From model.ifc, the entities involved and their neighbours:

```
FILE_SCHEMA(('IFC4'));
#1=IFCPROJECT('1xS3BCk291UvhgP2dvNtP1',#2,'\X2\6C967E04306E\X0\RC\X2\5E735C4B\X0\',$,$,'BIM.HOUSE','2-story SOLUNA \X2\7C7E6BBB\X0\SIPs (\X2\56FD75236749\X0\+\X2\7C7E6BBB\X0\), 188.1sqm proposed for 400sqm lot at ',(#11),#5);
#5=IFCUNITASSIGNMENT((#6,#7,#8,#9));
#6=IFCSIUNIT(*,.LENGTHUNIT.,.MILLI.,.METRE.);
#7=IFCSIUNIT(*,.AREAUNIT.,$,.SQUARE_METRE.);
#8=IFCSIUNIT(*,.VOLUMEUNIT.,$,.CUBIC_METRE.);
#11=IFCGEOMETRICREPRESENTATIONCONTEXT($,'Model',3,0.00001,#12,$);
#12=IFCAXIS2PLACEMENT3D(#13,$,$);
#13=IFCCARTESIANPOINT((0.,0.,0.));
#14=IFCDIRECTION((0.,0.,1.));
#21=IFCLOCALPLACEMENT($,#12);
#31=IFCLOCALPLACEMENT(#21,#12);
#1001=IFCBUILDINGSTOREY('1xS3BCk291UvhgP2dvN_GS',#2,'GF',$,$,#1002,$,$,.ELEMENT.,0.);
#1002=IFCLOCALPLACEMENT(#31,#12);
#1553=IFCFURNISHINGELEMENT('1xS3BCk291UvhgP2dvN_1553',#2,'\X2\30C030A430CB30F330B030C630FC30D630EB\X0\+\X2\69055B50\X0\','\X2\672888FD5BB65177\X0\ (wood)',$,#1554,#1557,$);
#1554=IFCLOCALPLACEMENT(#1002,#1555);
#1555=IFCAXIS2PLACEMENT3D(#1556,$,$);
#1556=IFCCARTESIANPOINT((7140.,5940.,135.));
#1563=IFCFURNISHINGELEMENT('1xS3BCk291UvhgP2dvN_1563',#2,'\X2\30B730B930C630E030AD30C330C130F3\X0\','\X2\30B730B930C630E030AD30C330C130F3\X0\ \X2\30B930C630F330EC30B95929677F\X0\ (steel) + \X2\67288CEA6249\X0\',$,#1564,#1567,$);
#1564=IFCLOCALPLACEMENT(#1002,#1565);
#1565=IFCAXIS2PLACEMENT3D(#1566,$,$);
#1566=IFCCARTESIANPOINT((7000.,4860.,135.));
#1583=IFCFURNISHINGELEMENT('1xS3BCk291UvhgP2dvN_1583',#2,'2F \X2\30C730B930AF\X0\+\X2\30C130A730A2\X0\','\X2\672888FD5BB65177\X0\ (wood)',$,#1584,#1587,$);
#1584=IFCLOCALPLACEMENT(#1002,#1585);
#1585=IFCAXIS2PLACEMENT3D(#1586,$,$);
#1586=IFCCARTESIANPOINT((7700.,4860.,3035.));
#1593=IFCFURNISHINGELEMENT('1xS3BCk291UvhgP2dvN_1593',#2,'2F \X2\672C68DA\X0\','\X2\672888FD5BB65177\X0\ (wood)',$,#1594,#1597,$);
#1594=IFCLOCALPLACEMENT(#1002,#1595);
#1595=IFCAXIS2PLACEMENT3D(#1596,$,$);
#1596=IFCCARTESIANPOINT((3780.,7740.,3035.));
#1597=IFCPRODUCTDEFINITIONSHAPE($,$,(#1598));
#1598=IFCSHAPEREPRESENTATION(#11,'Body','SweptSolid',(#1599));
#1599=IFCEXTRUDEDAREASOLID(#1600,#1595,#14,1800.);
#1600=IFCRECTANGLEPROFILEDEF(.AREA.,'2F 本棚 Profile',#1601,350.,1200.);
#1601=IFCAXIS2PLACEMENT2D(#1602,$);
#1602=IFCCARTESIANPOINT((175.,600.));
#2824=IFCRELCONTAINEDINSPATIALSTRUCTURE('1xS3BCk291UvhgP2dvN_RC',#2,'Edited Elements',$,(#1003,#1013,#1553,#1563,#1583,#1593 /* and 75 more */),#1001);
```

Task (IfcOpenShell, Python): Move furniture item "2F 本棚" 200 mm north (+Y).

```python
import ifcopenshell
import ifcopenshell.api.geometry
import ifcopenshell.util.placement
import ifcopenshell.util.unit

model = ifcopenshell.open("model.ifc")
unit_scale = ifcopenshell.util.unit.calculate_unit_scale(model)

item = model.by_guid("1xS3BCk291UvhgP2dvN_1593")
matrix = ifcopenshell.util.placement.get_local_placement(item.ObjectPlacement)
matrix[1, 3] += 0.2 / unit_scale
ifcopenshell.api.geometry.edit_object_placement(model, product=item, matrix=matrix, is_si=False)

print(ifcopenshell.util.placement.get_local_placement(item.ObjectPlacement).round(3) + 0.0)

model.write("model_updated.ifc")
```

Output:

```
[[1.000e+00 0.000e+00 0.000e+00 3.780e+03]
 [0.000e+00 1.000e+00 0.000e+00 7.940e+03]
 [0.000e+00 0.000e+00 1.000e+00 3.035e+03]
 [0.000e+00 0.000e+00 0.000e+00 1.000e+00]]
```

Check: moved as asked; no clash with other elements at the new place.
